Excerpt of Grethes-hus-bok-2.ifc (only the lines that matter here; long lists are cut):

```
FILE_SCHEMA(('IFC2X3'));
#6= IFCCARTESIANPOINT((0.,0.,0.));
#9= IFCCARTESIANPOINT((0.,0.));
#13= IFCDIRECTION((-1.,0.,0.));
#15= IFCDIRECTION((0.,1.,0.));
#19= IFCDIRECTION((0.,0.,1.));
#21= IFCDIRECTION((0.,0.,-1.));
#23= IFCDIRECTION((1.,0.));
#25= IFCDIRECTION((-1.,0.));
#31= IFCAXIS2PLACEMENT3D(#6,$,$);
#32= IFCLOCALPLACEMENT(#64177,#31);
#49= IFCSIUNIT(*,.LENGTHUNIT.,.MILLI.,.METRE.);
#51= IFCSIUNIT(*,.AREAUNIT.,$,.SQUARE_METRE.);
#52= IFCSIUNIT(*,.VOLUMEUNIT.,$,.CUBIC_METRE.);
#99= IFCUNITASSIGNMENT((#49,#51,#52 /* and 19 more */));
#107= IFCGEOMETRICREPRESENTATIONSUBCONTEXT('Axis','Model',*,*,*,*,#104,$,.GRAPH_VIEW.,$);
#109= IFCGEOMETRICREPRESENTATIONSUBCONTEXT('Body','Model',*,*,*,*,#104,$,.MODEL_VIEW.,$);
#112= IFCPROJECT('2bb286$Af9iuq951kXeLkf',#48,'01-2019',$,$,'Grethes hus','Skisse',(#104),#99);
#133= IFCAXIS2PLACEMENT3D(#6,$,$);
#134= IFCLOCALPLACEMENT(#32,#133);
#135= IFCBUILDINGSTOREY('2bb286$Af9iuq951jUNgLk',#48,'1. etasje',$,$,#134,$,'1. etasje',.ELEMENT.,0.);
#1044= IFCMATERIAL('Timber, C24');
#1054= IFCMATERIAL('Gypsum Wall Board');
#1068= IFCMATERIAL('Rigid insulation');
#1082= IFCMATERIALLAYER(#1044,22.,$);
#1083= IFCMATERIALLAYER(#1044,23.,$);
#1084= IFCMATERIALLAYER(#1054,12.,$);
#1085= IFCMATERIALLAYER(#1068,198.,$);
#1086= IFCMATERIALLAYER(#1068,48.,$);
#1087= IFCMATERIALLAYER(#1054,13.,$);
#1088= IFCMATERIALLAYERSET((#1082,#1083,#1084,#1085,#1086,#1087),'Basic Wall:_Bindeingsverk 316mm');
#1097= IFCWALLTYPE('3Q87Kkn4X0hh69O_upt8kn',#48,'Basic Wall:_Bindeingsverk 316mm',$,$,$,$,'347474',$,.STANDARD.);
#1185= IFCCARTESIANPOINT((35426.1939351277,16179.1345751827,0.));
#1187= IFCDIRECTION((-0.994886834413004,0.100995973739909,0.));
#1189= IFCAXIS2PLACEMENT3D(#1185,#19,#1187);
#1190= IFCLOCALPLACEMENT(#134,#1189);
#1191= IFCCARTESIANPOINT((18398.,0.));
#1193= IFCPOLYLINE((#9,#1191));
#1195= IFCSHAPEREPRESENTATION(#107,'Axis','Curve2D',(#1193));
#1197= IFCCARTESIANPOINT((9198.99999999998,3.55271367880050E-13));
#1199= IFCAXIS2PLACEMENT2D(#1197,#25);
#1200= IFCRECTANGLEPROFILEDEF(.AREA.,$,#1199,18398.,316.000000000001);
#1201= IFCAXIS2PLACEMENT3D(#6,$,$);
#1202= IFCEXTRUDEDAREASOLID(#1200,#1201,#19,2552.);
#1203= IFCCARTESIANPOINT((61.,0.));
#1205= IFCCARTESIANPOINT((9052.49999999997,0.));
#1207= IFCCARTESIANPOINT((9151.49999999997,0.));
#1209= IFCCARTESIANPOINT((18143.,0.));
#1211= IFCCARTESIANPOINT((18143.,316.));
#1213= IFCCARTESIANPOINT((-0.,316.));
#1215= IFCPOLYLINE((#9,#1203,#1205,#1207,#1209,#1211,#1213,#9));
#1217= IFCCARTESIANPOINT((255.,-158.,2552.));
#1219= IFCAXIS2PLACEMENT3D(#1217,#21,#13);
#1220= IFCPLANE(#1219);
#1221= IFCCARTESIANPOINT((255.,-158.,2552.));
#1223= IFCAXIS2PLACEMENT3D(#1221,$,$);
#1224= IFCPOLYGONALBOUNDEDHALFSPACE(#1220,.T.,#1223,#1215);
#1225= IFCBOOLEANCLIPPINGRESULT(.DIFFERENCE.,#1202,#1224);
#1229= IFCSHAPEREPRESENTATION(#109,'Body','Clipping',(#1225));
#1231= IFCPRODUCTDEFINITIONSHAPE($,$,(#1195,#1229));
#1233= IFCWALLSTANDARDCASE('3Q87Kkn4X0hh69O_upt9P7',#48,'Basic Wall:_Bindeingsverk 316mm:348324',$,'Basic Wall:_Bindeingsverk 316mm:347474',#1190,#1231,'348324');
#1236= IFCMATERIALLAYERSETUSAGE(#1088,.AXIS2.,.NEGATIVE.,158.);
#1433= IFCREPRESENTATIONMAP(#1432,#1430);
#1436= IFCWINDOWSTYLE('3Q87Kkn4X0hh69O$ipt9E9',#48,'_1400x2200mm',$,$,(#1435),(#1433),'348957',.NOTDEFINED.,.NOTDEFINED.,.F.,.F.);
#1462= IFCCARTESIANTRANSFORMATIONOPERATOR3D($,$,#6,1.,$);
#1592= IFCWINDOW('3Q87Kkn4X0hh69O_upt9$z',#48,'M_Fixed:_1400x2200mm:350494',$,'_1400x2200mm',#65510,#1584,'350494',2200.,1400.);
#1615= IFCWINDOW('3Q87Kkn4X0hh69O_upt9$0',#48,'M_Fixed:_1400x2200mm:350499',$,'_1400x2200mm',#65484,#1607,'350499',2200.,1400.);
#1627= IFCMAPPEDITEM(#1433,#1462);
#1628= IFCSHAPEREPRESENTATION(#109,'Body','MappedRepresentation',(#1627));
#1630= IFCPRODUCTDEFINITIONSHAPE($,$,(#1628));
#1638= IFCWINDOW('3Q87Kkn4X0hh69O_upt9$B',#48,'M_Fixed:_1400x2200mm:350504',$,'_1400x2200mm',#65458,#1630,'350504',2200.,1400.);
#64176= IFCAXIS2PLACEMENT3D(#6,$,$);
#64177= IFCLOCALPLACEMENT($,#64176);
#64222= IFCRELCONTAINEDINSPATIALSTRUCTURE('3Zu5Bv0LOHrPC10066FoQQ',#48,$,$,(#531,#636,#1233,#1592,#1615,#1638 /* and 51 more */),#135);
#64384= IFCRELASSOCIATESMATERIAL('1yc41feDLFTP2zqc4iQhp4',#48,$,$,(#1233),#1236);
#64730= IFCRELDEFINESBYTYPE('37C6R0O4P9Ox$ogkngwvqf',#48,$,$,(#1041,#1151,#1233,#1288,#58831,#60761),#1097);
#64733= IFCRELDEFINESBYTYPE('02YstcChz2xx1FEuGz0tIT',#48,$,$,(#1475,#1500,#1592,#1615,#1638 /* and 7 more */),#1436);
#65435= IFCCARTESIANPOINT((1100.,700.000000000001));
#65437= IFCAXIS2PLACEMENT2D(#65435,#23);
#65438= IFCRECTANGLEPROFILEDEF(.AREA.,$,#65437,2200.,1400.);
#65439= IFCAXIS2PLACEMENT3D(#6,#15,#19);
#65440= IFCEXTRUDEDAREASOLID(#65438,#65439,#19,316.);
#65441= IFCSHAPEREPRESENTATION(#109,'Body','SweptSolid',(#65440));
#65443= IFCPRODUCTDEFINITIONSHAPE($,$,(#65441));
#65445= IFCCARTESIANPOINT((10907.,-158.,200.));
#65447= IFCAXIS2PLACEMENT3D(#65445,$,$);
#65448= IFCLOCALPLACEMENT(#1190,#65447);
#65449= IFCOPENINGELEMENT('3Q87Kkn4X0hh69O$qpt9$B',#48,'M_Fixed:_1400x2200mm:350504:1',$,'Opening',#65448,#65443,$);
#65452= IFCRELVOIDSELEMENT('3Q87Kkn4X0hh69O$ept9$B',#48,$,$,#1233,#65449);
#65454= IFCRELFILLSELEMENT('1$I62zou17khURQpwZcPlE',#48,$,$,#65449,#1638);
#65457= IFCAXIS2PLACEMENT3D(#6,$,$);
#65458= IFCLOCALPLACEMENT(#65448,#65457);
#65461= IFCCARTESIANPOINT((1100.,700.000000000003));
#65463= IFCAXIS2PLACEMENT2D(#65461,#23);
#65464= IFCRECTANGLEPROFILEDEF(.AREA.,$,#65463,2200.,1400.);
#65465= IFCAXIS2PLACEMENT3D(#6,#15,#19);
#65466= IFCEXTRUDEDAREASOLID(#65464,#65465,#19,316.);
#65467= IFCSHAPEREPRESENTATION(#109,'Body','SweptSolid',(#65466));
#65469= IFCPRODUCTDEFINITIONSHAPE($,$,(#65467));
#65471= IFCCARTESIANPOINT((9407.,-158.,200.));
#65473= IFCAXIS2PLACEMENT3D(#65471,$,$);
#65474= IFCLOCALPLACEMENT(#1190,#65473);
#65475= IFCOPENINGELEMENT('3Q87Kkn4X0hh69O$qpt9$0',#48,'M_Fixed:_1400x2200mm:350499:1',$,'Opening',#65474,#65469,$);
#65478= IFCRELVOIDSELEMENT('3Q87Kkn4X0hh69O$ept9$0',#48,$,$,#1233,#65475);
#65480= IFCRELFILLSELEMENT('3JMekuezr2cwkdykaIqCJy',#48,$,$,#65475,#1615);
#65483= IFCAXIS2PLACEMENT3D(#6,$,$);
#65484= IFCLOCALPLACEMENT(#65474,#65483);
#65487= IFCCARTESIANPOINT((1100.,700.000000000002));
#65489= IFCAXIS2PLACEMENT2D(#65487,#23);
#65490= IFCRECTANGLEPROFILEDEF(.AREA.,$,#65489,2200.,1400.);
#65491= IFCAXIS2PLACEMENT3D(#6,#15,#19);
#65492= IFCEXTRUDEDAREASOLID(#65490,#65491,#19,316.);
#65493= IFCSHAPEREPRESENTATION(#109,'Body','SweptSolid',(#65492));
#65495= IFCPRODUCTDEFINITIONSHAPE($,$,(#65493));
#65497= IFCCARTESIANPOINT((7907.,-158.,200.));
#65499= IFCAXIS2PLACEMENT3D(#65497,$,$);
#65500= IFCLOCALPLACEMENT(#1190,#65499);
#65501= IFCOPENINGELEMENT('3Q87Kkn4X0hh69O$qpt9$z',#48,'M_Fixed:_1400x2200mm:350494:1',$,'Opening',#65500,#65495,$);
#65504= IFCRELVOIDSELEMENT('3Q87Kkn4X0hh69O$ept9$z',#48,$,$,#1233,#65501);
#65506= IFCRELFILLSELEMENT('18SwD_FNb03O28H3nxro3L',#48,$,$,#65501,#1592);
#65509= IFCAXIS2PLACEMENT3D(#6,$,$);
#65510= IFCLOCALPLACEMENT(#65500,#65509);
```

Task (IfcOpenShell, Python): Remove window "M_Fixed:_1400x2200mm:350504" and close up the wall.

```python
import ifcopenshell
import ifcopenshell.api.feature
import ifcopenshell.api.root
import ifcopenshell.geom
import ifcopenshell.util.shape

model = ifcopenshell.open("Grethes-hus-bok-2.ifc")
settings = ifcopenshell.geom.settings()


def volume(element):
    """Net volume in cubic metres, openings subtracted."""
    shape = ifcopenshell.geom.create_shape(settings, element)
    return ifcopenshell.util.shape.get_volume(shape.geometry)


window = model.by_guid("3Q87Kkn4X0hh69O_upt9$B")
opening = window.FillsVoids[0].RelatingOpeningElement
wall = opening.VoidsElements[0].RelatingBuildingElement
before = volume(wall)

ifcopenshell.api.root.remove_product(model, product=window)
ifcopenshell.api.feature.remove_feature(model, feature=opening)

after = volume(wall)

print(f"wall volume {before:.3f} -> {after:.3f} m3")

model.write("Grethes-hus-bok-2_updated.ifc")
```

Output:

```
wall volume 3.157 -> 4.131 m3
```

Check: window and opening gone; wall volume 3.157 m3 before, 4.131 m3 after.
